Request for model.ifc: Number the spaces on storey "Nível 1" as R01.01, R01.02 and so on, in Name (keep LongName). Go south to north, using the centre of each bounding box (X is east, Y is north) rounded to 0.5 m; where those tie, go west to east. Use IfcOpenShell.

First a look at what the model holds.

```python
import ifcopenshell
import ifcopenshell.util.element
import ifcopenshell.util.placement

model = ifcopenshell.open("model.ifc")
print(model.schema)
storey = next(s for s in model.by_type("IfcBuildingStorey") if s.Name == "Nível 1")
spaces = [e for e in ifcopenshell.util.element.get_decomposition(storey) if e.is_a("IfcSpace")]
for e in sorted(spaces, key=lambda e: e.id()):
    origin = ifcopenshell.util.placement.get_local_placement(e.ObjectPlacement)[:3, 3]
    print(e.id(), e.Name, e.LongName, origin.round(2) + 0.0, sep=" | ")
```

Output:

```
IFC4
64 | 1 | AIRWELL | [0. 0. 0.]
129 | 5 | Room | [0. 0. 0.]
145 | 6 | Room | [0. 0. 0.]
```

```python
import ifcopenshell
import ifcopenshell.geom
import ifcopenshell.util.element
import ifcopenshell.util.shape

model = ifcopenshell.open("model.ifc")
settings = ifcopenshell.geom.settings()
settings.set("use-world-coords", True)


def centre(element):
    shape = ifcopenshell.geom.create_shape(settings, element)
    return ifcopenshell.util.shape.get_bbox_centroid(shape.geometry)


storey = next(s for s in model.by_type("IfcBuildingStorey") if s.Name == "Nível 1")
spaces = [e for e in ifcopenshell.util.element.get_decomposition(storey) if e.is_a("IfcSpace")]

# Insertion points can sit at a corner or the storey origin, so sort by the geometry (in metres).
centres = {e: centre(e) for e in spaces}
spaces.sort(key=lambda e: (round(centres[e][1] / 0.5), centres[e][0]))

for i, e in enumerate(spaces, start=1):
    number = f"R01.{i:02d}"
    e.Name = number
    print(e.id(), number)

model.write("model_rev.ifc")
```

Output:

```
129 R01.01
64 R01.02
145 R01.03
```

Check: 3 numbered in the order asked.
